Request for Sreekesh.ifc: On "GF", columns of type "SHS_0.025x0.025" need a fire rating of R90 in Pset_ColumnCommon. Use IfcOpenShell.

First a look at what the model holds.

```python
import ifcopenshell
import ifcopenshell.util.element

model = ifcopenshell.open("Sreekesh.ifc")
print(model.schema)
storey = next(s for s in model.by_type("IfcBuildingStorey") if s.Name == "GF")
columns = [e for e in ifcopenshell.util.element.get_decomposition(storey) if e.is_a("IfcColumn")]
seen = {}
for e in columns:
    element_type = ifcopenshell.util.element.get_type(e)
    key = (element_type.Name if element_type != e and element_type else None, ifcopenshell.util.element.get_pset(e, "Pset_ColumnCommon", "FireRating"))
    seen[key] = seen.get(key, 0) + 1
for (name, value), count in sorted(seen.items(), key=str):
    print(count, "x", name, "|", value)
```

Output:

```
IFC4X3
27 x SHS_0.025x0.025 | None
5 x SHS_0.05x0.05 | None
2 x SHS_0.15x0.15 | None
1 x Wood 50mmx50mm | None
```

```python
import ifcopenshell
import ifcopenshell.api.pset
import ifcopenshell.util.element

model = ifcopenshell.open("Sreekesh.ifc")

storey = next(s for s in model.by_type("IfcBuildingStorey") if s.Name == "GF")
columns = [e for e in ifcopenshell.util.element.get_decomposition(storey) if e.is_a("IfcColumn")]

count = 0
for e in columns:
    element_type = ifcopenshell.util.element.get_type(e)
    if element_type in (None, e) or element_type.Name != "SHS_0.025x0.025":
        continue
    # add_pset returns the element's existing set when there is one.
    pset = ifcopenshell.api.pset.add_pset(model, product=e, name="Pset_ColumnCommon")
    ifcopenshell.api.pset.edit_pset(model, pset=pset, properties={"FireRating": "R90"})
    count += 1

print(count, "columns updated")

model.write("Sreekesh-out.ifc")
```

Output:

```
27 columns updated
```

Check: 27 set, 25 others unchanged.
